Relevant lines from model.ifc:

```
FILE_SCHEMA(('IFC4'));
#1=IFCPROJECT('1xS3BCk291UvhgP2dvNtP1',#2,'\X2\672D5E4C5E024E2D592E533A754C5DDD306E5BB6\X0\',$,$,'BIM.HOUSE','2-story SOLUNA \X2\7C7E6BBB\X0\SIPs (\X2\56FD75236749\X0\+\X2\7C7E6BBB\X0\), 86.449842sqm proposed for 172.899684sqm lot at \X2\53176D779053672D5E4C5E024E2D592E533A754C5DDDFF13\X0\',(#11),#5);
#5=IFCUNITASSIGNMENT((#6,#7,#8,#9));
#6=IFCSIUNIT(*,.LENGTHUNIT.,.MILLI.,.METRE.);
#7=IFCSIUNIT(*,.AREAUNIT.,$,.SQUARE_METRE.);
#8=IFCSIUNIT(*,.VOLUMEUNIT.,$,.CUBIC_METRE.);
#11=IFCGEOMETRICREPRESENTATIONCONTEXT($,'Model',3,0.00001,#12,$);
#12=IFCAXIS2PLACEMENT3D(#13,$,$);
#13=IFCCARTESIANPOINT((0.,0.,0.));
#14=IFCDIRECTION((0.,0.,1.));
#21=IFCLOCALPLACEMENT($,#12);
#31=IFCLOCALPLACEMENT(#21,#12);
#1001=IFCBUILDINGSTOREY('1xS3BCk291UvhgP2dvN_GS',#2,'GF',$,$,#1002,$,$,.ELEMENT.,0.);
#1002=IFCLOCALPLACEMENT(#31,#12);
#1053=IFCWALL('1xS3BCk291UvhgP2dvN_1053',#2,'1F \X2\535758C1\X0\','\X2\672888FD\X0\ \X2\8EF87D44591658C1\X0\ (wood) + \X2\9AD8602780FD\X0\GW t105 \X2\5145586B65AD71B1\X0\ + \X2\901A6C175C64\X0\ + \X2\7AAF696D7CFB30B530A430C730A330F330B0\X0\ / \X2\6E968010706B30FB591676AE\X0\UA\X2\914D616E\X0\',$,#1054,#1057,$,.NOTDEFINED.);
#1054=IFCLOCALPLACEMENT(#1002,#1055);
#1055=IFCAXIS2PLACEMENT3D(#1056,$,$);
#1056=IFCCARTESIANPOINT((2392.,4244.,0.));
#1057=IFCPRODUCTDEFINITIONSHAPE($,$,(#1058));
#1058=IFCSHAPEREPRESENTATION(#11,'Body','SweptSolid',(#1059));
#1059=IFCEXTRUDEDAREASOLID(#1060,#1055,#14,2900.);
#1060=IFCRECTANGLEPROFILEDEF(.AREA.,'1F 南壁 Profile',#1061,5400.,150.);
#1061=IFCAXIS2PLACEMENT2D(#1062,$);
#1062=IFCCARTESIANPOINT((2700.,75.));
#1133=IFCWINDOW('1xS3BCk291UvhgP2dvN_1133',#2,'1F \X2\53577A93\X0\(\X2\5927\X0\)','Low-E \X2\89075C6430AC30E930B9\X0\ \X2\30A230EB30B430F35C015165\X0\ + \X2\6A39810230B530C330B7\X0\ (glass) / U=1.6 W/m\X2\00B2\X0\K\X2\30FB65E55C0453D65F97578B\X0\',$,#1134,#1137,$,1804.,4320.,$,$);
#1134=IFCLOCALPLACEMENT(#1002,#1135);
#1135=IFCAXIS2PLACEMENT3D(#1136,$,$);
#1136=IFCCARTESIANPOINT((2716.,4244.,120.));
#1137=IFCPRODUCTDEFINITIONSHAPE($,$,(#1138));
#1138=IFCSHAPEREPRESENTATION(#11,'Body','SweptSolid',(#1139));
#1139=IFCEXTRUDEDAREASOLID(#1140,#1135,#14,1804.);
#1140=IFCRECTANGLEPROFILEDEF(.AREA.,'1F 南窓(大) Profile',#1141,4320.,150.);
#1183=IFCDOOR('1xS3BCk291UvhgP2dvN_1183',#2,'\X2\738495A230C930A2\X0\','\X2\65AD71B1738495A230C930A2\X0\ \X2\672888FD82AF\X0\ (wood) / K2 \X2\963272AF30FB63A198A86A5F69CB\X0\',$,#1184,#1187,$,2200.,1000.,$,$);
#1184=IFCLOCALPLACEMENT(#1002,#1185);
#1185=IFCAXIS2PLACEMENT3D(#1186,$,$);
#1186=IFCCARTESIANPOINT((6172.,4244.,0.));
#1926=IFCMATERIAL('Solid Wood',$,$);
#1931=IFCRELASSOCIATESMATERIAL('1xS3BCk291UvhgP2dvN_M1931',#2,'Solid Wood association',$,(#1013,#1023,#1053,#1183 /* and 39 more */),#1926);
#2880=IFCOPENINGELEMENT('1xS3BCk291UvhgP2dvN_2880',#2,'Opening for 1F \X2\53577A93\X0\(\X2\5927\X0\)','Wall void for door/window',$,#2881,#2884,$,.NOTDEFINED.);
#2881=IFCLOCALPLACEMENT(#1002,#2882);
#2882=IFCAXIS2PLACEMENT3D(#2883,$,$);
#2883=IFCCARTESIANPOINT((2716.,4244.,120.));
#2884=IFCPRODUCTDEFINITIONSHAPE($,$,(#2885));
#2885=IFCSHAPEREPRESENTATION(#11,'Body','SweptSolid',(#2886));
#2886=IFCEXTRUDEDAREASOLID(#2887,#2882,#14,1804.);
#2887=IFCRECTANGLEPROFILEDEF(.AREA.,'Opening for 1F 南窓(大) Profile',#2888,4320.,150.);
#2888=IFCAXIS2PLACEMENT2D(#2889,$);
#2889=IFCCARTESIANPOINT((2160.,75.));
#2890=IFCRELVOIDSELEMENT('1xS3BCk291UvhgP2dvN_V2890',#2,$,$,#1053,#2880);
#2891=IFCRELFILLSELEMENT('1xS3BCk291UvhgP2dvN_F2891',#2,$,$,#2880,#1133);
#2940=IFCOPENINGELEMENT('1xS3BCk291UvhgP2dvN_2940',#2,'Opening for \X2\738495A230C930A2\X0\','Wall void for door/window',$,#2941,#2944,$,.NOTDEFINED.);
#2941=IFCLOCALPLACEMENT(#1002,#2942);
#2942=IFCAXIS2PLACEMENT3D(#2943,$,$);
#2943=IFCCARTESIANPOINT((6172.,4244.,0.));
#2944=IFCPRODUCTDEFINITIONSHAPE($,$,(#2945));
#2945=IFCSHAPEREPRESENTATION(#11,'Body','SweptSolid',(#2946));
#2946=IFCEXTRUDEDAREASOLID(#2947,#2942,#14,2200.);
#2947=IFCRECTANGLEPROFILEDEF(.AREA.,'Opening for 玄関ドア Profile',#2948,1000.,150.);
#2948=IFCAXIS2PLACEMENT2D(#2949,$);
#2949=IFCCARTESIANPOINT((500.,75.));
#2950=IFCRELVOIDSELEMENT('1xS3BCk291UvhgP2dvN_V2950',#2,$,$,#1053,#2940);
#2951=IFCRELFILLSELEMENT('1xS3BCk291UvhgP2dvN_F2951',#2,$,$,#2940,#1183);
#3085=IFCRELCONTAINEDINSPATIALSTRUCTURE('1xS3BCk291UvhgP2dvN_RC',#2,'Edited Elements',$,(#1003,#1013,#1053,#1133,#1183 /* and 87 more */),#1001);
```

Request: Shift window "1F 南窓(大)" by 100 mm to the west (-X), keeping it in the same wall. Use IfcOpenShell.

```python
import ifcopenshell
import ifcopenshell.api.geometry
import ifcopenshell.util.placement

model = ifcopenshell.open("model.ifc")

window = model.by_guid("1xS3BCk291UvhgP2dvN_1133")
opening = window.FillsVoids[0].RelatingOpeningElement
wall = opening.VoidsElements[0].RelatingBuildingElement

wall_matrix = ifcopenshell.util.placement.get_local_placement(wall.ObjectPlacement)
shift = wall_matrix[:3, 0] * -100.0
before = ifcopenshell.util.placement.get_local_placement(window.ObjectPlacement)[:3, 3].copy()

# The window is not placed relative to its opening, so move both.
for product in (opening, window):
    matrix = ifcopenshell.util.placement.get_local_placement(product.ObjectPlacement)
    matrix[:3, 3] += shift
    ifcopenshell.api.geometry.edit_object_placement(model, product=product, matrix=matrix, is_si=False)

after = ifcopenshell.util.placement.get_local_placement(window.ObjectPlacement)[:3, 3]
print("window moved by", (after - before).round(3) + 0.0)

model.write("model_rev.ifc")
```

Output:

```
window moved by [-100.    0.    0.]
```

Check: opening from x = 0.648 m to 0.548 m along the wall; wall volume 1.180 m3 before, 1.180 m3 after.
